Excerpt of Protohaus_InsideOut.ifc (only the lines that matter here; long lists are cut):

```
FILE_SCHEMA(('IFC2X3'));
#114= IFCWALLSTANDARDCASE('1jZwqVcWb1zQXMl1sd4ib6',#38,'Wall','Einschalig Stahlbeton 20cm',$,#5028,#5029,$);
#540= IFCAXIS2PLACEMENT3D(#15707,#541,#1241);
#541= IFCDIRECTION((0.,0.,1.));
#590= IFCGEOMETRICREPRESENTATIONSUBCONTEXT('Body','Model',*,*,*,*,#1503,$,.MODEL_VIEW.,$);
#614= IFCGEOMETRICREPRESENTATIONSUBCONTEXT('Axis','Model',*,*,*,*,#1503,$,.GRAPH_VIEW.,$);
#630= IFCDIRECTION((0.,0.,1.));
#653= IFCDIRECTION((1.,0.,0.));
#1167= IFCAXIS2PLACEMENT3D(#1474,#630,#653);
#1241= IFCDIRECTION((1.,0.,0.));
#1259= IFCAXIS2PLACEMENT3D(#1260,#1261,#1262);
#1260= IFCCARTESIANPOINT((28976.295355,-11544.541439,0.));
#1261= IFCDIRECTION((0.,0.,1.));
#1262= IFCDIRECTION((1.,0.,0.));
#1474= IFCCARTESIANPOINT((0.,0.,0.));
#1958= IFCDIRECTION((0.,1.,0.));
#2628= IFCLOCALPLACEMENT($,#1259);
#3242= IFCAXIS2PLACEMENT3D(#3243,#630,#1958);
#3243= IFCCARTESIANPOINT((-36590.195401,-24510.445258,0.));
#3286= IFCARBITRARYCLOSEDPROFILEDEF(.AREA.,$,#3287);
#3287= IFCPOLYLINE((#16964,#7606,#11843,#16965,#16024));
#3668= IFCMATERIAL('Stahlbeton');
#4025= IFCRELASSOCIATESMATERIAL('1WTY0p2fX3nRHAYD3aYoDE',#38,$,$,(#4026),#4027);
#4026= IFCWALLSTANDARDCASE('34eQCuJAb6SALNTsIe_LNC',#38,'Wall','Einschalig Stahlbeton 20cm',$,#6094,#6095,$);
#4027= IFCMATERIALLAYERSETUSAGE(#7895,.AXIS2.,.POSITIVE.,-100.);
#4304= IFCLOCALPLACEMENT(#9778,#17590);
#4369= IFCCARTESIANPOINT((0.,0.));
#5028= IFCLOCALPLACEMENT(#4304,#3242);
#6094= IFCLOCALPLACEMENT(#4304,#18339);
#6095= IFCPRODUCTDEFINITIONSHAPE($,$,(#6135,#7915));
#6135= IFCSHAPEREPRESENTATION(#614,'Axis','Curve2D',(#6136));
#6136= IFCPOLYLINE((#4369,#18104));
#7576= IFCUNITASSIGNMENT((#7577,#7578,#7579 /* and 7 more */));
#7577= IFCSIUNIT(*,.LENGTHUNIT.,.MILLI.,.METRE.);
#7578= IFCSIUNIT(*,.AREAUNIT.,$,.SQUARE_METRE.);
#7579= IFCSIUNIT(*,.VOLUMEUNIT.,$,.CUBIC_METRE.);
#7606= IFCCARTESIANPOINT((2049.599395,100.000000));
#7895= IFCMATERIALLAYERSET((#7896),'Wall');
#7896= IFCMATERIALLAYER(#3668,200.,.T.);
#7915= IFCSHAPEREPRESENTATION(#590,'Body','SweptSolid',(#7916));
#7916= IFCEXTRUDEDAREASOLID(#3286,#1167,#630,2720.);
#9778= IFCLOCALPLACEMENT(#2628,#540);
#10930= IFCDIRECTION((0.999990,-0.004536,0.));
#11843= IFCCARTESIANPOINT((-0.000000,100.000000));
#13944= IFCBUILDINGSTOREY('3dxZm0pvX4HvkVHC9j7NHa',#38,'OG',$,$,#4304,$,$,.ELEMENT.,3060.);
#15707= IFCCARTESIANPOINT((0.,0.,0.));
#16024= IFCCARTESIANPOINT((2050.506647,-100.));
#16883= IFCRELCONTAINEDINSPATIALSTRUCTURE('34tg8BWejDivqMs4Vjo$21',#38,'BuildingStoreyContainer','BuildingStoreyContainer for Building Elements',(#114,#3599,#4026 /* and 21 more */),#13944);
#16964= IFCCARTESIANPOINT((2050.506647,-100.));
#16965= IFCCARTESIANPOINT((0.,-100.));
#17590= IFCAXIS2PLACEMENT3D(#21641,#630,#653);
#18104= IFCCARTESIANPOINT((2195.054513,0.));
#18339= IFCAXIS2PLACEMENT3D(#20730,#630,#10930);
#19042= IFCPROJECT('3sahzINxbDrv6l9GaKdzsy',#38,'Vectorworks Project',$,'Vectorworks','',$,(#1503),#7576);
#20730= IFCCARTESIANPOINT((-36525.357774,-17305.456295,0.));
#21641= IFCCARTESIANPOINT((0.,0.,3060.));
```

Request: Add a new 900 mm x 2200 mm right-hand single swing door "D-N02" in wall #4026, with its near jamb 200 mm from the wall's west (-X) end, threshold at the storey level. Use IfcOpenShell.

```python
import numpy as np
import ifcopenshell
import ifcopenshell.api.feature
import ifcopenshell.api.geometry
import ifcopenshell.api.root
import ifcopenshell.api.spatial
import ifcopenshell.api.type
import ifcopenshell.geom
import ifcopenshell.util.element
import ifcopenshell.util.placement
import ifcopenshell.util.representation
import ifcopenshell.util.shape
import ifcopenshell.util.unit

model = ifcopenshell.open("Protohaus_InsideOut.ifc")
unit_scale = ifcopenshell.util.unit.calculate_unit_scale(model)
settings = ifcopenshell.geom.settings()


def volume(element):
    """Net volume in cubic metres, openings subtracted."""
    shape = ifcopenshell.geom.create_shape(settings, element)
    return ifcopenshell.util.shape.get_volume(shape.geometry)


wall = model.by_id(4026)
storey = ifcopenshell.util.element.get_container(wall, ifc_class="IfcBuildingStorey")
context = ifcopenshell.util.representation.get_context(model, "Model", "Body", "MODEL_VIEW")
before = volume(wall)

width, height, from_end, sill = 0.9, 2.2, 0.2, 0.0  # metres

# The wall runs along its own X axis, and the end named is its -X end.
wall_shape = ifcopenshell.geom.create_shape(settings, wall)
x, y, z = ifcopenshell.util.shape.get_vertices(wall_shape.geometry).T
start = x.min() + from_end
face, thickness = float(y.min()), float(y.max() - y.min())
wall_matrix = ifcopenshell.util.placement.get_local_placement(wall.ObjectPlacement)
level = ifcopenshell.util.placement.get_local_placement(storey.ObjectPlacement)[2, 3]


def in_wall(x, y):
    """Placement at x, y metres in the wall's axes, at sill height."""
    matrix = wall_matrix.copy()
    matrix[:, 3] = wall_matrix @ np.array([x / unit_scale, y / unit_scale, 0.0, 1.0])
    matrix[2, 3] = level + sill / unit_scale
    return matrix


# Opening: a box that overshoots both wall faces by 50 mm.
opening = ifcopenshell.api.root.create_entity(model, ifc_class="IfcOpeningElement")
box = ifcopenshell.api.geometry.add_wall_representation(
    model, context=context, length=width, height=height, thickness=thickness + 0.1
)
ifcopenshell.api.geometry.assign_representation(model, product=opening, representation=box)
ifcopenshell.api.geometry.edit_object_placement(model, product=opening, matrix=in_wall(start, face - 0.05), is_si=False)
ifcopenshell.api.feature.add_feature(model, feature=opening, element=wall)

door = ifcopenshell.api.root.create_entity(model, ifc_class="IfcDoor", name="D-N02")
door.OverallWidth, door.OverallHeight = width / unit_scale, height / unit_scale
body = ifcopenshell.api.geometry.add_door_representation(
    model,
    context=context,
    overall_width=door.OverallWidth,
    overall_height=door.OverallHeight,
    operation_type="SINGLE_SWING_RIGHT",
    lining_properties={"LiningDepth": thickness / unit_scale, "ThresholdDepth": thickness / unit_scale},
)
ifcopenshell.api.geometry.assign_representation(model, product=door, representation=body)
ifcopenshell.api.spatial.assign_container(model, products=[door], relating_structure=storey)
fills = ifcopenshell.api.feature.add_filling(model, opening=opening, element=door)
fills.OwnerHistory = door.OwnerHistory  # required in IFC2X3

# IFC2X3 keeps the operation on the door style.
style = ifcopenshell.api.root.create_entity(model, ifc_class="IfcDoorStyle", name="D-N02")
style.OperationType, style.ConstructionType = "SINGLE_SWING_RIGHT", "NOTDEFINED"
style.ParameterTakesPrecedence = style.Sizeable = False
ifcopenshell.api.type.assign_type(model, related_objects=[door], relating_type=style)

# The lining spans the wall, so the door starts at the wall face.
ifcopenshell.api.geometry.edit_object_placement(model, product=door, matrix=in_wall(start, face), is_si=False)

after = volume(wall)

print(f"wall volume {before:.3f} -> {after:.3f} m3")

model.write("Protohaus_InsideOut_v2.ifc")
```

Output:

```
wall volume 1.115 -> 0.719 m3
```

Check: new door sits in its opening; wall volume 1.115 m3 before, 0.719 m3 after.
